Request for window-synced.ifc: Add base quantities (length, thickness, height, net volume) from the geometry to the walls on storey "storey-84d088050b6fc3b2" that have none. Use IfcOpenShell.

First a look at what the model holds.

```python
import ifcopenshell
import ifcopenshell.util.element
import ifcopenshell.util.unit

model = ifcopenshell.open("window-synced.ifc")
print(model.schema)
for unit_type in ("LENGTHUNIT", "AREAUNIT", "VOLUMEUNIT"):
    print(unit_type, ifcopenshell.util.unit.calculate_unit_scale(model, unit_type))
storey = next(s for s in model.by_type("IfcBuildingStorey") if s.Name == "storey-84d088050b6fc3b2")
walls = [e for e in ifcopenshell.util.element.get_decomposition(storey) if e.is_a("IfcWall")]
for e in sorted(walls, key=lambda e: e.id()):
    print(e.id(), e.is_a(), e.Name, list(ifcopenshell.util.element.get_psets(e, qtos_only=True)), sep=" | ")
```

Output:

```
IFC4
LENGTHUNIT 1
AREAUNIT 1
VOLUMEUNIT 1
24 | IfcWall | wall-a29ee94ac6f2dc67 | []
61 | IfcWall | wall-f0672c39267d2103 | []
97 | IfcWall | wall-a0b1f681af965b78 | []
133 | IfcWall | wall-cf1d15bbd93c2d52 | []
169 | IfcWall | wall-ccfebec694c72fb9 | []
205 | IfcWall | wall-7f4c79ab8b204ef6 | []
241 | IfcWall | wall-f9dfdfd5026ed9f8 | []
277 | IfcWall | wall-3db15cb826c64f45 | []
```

```python
import ifcopenshell
import ifcopenshell.api.pset
import ifcopenshell.geom
import ifcopenshell.util.element
import ifcopenshell.util.shape
import ifcopenshell.util.unit

model = ifcopenshell.open("window-synced.ifc")
unit_scale = ifcopenshell.util.unit.calculate_unit_scale(model)
volume_scale = ifcopenshell.util.unit.calculate_unit_scale(model, "VOLUMEUNIT")
settings = ifcopenshell.geom.settings()

storey = next(s for s in model.by_type("IfcBuildingStorey") if s.Name == "storey-84d088050b6fc3b2")
walls = [e for e in ifcopenshell.util.element.get_decomposition(storey) if e.is_a("IfcWall")]

for e in sorted(walls, key=lambda e: e.id()):
    if ifcopenshell.util.element.get_psets(e, qtos_only=True, should_inherit=False):
        continue
    # Geometry comes back in metres, in the element's own axes.
    shape = ifcopenshell.geom.create_shape(settings, e)
    values = {
        "Length": ifcopenshell.util.shape.get_x(shape.geometry) / unit_scale,
        "Width": ifcopenshell.util.shape.get_y(shape.geometry) / unit_scale,
        "Height": ifcopenshell.util.shape.get_z(shape.geometry) / unit_scale,
        "NetVolume": ifcopenshell.util.shape.get_volume(shape.geometry) / volume_scale,
    }
    qto = ifcopenshell.api.pset.add_qto(model, product=e, name="Qto_WallBaseQuantities")
    ifcopenshell.api.pset.edit_qto(model, qto=qto, properties=values)
    print(e.id(), {k: round(v, 3) for k, v in values.items()})

model.write("window-synced-out.ifc")
```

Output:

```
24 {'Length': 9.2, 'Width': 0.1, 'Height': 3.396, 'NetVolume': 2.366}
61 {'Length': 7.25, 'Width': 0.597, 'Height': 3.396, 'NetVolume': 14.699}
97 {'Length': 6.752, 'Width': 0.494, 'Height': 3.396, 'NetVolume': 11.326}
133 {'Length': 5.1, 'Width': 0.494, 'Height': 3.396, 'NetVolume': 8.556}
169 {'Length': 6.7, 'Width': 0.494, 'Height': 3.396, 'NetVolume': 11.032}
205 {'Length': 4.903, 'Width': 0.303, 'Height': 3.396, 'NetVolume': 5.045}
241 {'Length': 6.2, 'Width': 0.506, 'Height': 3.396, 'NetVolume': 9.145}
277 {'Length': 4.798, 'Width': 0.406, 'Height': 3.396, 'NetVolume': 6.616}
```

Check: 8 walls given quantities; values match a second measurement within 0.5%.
